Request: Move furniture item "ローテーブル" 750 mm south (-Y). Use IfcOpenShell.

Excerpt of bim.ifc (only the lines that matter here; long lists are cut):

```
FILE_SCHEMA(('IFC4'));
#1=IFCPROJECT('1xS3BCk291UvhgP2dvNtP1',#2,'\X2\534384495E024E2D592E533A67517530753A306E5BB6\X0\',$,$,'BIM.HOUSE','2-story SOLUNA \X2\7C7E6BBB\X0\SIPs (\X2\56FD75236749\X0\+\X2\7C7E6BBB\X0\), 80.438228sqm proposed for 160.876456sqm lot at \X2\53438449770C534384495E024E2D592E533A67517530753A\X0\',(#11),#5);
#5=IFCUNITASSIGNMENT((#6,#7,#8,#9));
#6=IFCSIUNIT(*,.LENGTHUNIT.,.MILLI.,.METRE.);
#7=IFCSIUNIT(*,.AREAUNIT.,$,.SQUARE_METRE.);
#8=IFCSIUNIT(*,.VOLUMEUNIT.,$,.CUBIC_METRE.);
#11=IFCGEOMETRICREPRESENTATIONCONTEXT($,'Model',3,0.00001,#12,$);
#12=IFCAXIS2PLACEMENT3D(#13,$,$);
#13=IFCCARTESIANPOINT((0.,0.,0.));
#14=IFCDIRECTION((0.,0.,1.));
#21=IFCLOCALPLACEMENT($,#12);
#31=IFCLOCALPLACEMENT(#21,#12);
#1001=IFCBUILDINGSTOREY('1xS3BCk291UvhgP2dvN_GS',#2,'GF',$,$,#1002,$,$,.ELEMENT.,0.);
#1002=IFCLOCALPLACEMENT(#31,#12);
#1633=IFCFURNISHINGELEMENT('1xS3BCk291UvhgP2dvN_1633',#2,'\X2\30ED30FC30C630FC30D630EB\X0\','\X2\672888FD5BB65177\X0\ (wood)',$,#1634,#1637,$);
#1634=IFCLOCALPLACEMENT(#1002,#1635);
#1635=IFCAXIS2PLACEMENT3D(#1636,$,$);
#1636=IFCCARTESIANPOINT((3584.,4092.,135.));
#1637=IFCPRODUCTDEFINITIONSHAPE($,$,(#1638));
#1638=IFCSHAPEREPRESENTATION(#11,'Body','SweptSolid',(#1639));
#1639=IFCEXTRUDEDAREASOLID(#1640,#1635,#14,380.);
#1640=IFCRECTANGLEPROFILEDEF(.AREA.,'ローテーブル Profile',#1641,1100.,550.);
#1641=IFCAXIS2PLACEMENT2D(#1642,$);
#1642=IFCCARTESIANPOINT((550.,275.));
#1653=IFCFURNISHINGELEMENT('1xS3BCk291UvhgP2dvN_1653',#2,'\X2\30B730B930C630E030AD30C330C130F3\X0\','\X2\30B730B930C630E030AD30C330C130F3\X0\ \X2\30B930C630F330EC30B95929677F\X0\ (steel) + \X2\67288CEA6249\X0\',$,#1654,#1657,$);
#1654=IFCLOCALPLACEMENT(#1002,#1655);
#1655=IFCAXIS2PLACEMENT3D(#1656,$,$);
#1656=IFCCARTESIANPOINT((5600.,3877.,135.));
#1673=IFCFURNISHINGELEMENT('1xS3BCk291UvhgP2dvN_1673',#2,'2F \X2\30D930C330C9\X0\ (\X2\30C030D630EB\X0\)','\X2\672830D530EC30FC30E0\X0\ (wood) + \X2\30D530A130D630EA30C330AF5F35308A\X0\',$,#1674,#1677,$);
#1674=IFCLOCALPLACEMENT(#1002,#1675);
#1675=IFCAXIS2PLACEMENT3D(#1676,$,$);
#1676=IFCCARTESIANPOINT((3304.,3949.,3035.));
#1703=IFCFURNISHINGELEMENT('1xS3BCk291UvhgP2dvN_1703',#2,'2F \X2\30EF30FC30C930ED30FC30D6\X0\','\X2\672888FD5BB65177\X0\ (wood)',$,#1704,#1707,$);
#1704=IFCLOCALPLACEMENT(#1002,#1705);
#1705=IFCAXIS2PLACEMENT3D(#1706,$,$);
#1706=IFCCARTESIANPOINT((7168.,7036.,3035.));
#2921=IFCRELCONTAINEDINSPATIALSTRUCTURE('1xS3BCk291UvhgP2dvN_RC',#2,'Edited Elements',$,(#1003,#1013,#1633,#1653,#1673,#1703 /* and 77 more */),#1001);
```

```python
import ifcopenshell
import ifcopenshell.api.geometry
import ifcopenshell.util.placement
import ifcopenshell.util.unit

model = ifcopenshell.open("bim.ifc")
unit_scale = ifcopenshell.util.unit.calculate_unit_scale(model)

item = model.by_guid("1xS3BCk291UvhgP2dvN_1633")
matrix = ifcopenshell.util.placement.get_local_placement(item.ObjectPlacement)
matrix[1, 3] -= 0.75 / unit_scale
ifcopenshell.api.geometry.edit_object_placement(model, product=item, matrix=matrix, is_si=False)

print(ifcopenshell.util.placement.get_local_placement(item.ObjectPlacement).round(3) + 0.0)

model.write("bim_rev.ifc")
```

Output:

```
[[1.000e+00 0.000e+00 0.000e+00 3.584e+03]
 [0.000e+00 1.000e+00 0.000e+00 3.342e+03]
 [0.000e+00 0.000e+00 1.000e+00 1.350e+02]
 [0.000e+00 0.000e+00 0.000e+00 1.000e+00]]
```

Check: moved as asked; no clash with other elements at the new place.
